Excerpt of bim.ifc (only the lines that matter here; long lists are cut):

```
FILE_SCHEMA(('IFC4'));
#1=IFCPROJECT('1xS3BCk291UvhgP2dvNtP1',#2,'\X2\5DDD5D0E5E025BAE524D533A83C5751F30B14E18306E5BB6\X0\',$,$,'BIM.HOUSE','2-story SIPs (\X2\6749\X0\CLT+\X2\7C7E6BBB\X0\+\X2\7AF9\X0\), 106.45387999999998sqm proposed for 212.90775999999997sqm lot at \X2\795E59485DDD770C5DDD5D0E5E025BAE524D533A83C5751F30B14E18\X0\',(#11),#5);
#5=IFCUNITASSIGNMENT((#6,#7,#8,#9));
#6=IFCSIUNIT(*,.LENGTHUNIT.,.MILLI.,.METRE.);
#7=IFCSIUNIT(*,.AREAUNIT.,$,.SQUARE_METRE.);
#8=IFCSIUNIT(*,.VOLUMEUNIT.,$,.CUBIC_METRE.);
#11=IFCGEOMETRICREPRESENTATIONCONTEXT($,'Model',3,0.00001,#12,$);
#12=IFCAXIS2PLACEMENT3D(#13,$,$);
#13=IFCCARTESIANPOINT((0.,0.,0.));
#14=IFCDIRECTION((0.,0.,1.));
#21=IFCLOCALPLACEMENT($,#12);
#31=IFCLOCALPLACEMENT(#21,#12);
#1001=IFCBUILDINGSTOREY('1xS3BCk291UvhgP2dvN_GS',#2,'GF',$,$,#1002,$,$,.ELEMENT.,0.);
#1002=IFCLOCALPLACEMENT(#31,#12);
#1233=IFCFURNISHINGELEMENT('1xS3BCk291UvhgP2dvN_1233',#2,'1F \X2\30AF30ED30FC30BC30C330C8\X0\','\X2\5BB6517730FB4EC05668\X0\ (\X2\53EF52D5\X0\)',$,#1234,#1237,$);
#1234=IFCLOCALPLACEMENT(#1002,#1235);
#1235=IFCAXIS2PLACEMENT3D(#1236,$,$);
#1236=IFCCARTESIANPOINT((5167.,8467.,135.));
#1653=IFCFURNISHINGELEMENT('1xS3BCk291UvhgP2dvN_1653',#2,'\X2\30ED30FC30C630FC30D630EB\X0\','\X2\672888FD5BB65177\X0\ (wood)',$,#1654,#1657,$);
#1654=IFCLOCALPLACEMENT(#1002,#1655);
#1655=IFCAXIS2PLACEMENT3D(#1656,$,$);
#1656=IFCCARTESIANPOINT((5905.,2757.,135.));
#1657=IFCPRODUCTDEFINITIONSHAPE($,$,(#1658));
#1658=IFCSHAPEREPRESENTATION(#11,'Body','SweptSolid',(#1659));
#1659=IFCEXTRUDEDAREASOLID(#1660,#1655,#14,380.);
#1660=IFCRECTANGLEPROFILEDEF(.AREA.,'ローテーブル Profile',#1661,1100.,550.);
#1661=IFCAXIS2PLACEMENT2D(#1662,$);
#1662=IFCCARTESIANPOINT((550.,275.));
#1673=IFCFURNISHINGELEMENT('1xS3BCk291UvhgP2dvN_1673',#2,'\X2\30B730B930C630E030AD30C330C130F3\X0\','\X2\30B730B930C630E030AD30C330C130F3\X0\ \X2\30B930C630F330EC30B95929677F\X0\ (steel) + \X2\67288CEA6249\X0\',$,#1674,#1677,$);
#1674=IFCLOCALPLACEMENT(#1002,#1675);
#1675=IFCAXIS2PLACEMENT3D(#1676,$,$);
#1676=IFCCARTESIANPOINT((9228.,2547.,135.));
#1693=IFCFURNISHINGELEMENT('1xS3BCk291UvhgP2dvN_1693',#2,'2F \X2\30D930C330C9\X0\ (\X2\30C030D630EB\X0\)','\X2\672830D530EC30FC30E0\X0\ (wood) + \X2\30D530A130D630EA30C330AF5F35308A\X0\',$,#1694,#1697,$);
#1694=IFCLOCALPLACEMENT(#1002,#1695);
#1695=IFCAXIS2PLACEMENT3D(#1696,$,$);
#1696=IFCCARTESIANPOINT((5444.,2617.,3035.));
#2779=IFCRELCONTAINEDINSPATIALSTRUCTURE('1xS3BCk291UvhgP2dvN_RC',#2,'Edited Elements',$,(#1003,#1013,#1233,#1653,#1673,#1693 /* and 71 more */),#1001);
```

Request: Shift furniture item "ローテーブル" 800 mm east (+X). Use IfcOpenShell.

```python
import ifcopenshell
import ifcopenshell.api.geometry
import ifcopenshell.util.placement
import ifcopenshell.util.unit

model = ifcopenshell.open("bim.ifc")
unit_scale = ifcopenshell.util.unit.calculate_unit_scale(model)

item = model.by_id(1653)
matrix = ifcopenshell.util.placement.get_local_placement(item.ObjectPlacement)
matrix[0, 3] += 0.8 / unit_scale
ifcopenshell.api.geometry.edit_object_placement(model, product=item, matrix=matrix, is_si=False)

print(ifcopenshell.util.placement.get_local_placement(item.ObjectPlacement).round(3) + 0.0)

model.write("bim_updated.ifc")
```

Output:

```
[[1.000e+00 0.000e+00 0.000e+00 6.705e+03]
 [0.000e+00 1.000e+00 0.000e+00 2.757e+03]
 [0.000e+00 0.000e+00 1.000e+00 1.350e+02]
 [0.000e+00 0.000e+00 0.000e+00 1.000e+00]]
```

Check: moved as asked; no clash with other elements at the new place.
